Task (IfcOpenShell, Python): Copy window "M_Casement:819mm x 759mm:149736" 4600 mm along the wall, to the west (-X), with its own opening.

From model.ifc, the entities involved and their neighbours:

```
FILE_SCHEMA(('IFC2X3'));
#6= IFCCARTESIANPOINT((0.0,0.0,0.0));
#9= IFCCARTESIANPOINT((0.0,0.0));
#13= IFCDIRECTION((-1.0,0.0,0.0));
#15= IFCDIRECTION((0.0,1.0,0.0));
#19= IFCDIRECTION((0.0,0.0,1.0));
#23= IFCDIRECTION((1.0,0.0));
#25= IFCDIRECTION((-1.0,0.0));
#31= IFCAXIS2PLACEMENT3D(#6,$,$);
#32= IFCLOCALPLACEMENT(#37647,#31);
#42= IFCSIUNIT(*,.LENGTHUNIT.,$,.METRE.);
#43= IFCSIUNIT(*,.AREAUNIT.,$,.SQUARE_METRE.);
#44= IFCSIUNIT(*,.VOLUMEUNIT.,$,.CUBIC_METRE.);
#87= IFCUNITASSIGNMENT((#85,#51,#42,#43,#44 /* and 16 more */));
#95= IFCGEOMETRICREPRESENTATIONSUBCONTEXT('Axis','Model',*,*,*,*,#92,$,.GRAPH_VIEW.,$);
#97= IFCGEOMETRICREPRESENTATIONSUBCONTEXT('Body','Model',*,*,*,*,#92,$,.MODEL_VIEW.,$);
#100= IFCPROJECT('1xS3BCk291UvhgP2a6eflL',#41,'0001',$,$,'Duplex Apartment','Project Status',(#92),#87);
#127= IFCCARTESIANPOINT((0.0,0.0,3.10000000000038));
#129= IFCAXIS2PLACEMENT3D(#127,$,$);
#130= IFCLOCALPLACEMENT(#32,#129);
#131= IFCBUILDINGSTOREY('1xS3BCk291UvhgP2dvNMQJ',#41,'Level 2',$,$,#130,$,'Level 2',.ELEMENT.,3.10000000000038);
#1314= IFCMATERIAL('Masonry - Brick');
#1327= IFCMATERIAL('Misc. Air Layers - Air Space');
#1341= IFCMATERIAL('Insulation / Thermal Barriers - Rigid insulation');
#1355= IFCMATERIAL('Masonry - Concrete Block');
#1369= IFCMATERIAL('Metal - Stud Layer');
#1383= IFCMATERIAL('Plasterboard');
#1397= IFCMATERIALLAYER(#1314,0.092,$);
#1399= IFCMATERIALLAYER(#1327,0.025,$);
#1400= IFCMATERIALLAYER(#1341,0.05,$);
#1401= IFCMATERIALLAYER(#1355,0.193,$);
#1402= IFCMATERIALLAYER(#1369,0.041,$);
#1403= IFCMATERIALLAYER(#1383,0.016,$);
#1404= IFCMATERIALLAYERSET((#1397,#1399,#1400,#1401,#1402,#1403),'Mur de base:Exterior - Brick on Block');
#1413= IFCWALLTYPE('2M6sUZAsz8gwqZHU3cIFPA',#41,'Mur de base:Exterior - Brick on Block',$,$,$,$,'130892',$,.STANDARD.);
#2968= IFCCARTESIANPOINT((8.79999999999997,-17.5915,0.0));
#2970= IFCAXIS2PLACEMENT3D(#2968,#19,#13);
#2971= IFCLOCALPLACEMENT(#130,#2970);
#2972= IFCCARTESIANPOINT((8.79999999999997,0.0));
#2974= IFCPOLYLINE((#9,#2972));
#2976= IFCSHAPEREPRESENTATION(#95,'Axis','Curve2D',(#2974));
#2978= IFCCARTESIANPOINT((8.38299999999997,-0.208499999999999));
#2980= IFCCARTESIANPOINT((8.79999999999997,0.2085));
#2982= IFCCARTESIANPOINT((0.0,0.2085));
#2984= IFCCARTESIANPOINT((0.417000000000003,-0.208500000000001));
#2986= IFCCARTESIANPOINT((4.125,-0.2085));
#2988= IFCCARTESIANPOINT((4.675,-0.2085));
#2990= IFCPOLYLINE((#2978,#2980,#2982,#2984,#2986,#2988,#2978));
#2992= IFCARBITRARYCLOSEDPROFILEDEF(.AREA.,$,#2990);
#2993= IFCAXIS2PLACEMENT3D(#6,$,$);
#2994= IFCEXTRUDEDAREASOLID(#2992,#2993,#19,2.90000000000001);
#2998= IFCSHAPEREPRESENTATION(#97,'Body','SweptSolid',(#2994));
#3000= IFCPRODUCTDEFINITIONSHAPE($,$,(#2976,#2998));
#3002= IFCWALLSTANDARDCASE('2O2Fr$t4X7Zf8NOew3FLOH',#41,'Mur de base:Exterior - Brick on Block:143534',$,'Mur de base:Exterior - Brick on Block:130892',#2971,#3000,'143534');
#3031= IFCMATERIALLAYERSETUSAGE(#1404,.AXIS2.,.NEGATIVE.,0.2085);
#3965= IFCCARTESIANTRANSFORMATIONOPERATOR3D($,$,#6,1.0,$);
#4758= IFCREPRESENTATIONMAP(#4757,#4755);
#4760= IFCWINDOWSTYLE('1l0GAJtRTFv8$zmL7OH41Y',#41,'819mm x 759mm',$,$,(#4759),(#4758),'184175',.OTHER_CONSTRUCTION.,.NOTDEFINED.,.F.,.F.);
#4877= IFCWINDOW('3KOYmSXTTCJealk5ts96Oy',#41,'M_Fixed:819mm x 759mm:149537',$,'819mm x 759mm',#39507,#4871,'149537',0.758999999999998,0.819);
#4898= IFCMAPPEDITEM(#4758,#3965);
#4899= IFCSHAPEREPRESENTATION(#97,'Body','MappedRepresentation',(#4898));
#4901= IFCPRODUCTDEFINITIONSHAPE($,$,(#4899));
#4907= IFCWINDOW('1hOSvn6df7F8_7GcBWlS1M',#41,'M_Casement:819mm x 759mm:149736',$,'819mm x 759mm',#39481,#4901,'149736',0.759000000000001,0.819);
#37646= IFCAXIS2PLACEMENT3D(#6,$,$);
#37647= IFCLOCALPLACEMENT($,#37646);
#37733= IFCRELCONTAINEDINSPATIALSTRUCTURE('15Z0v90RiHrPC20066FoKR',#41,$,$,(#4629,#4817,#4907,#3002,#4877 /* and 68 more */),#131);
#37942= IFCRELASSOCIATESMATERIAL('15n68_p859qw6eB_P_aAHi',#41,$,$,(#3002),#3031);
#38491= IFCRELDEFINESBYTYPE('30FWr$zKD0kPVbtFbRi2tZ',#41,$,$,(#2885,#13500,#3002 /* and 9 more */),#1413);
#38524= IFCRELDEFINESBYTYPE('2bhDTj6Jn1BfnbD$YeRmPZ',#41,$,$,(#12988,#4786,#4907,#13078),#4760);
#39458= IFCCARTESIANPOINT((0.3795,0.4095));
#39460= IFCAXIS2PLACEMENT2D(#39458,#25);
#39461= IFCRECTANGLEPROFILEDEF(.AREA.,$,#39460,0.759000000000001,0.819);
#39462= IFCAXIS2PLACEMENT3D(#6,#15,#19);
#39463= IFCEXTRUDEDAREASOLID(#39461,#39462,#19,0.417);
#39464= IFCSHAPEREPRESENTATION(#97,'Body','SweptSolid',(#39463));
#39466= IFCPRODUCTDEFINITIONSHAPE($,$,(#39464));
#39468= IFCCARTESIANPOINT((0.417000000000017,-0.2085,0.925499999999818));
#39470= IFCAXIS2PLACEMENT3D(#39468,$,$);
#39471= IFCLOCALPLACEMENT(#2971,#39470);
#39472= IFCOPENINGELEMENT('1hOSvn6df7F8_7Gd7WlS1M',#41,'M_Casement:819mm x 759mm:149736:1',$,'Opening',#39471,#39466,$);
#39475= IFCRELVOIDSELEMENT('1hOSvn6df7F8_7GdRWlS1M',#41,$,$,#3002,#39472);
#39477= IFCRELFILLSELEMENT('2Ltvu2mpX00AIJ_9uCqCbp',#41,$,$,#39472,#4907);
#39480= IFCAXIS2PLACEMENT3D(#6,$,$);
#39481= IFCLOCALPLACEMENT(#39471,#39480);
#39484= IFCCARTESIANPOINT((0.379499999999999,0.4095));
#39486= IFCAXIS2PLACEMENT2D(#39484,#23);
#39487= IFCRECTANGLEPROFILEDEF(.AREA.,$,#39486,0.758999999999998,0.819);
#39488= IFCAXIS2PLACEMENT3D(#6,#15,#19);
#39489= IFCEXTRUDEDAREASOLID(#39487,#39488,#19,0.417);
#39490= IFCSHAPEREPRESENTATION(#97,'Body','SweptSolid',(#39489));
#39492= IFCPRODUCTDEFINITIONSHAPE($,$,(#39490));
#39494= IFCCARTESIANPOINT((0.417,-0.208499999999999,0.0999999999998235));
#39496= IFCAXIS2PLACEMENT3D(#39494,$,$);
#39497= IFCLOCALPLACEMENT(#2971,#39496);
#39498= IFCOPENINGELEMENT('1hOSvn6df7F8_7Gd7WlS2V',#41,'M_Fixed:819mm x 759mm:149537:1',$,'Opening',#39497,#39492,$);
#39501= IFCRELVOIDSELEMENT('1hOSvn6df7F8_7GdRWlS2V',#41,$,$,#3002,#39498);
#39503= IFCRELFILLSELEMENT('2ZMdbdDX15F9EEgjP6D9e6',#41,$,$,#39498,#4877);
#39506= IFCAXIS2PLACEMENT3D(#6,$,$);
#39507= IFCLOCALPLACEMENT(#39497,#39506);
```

```python
import ifcopenshell
import ifcopenshell.api.feature
import ifcopenshell.api.geometry
import ifcopenshell.api.root
import ifcopenshell.geom
import ifcopenshell.util.element
import ifcopenshell.util.placement
import ifcopenshell.util.shape
import ifcopenshell.util.unit

model = ifcopenshell.open("model.ifc")
unit_scale = ifcopenshell.util.unit.calculate_unit_scale(model)
settings = ifcopenshell.geom.settings()


def volume(element):
    """Net volume in cubic metres, openings subtracted."""
    shape = ifcopenshell.geom.create_shape(settings, element)
    return ifcopenshell.util.shape.get_volume(shape.geometry)


def reuse_history(source, copy):
    """copy_class also copies each property set's owner history, people and application; keep the originals."""
    for rel in copy.IsDefinedBy:
        if rel.is_a("IfcRelDefinesByProperties") and (history := rel.RelatingPropertyDefinition.OwnerHistory):
            rel.RelatingPropertyDefinition.OwnerHistory = source.OwnerHistory
            ifcopenshell.util.element.remove_deep2(model, history)


window = model.by_guid("1hOSvn6df7F8_7GcBWlS1M")
opening = window.FillsVoids[0].RelatingOpeningElement
wall = opening.VoidsElements[0].RelatingBuildingElement
before = volume(wall)
shift = ifcopenshell.util.placement.get_local_placement(wall.ObjectPlacement)[:3, 0] * 4.6 / unit_scale

# copy_class copies the void relationship, type, container and properties, but no geometry.
new_opening = ifcopenshell.api.root.copy_class(model, product=opening)
new_opening.Representation = ifcopenshell.util.element.copy_deep(
    model, opening.Representation, exclude=["IfcGeometricRepresentationContext", "IfcRepresentationMap"]
)
new_opening.Name = "M_Casement:819mm x 759mm"
new_window = ifcopenshell.api.root.copy_class(model, product=window)
new_window.Representation = ifcopenshell.util.element.copy_deep(
    model, window.Representation, exclude=["IfcGeometricRepresentationContext", "IfcRepresentationMap"]
)
new_window.Name = "M_Casement:819mm x 759mm"
new_window.Tag = None
reuse_history(window, new_window)
fills = ifcopenshell.api.feature.add_filling(model, opening=new_opening, element=new_window)
fills.OwnerHistory = new_window.OwnerHistory  # required in IFC2X3

for old, new in ((opening, new_opening), (window, new_window)):
    matrix = ifcopenshell.util.placement.get_local_placement(old.ObjectPlacement)
    matrix[:3, 3] += shift
    ifcopenshell.api.geometry.edit_object_placement(model, product=new, matrix=matrix, is_si=False)

after = volume(wall)

print(f"wall volume {before:.3f} -> {after:.3f} m3")

model.write("model_v2.ifc")
```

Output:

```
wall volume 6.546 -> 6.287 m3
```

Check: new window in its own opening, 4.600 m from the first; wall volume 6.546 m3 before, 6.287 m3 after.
